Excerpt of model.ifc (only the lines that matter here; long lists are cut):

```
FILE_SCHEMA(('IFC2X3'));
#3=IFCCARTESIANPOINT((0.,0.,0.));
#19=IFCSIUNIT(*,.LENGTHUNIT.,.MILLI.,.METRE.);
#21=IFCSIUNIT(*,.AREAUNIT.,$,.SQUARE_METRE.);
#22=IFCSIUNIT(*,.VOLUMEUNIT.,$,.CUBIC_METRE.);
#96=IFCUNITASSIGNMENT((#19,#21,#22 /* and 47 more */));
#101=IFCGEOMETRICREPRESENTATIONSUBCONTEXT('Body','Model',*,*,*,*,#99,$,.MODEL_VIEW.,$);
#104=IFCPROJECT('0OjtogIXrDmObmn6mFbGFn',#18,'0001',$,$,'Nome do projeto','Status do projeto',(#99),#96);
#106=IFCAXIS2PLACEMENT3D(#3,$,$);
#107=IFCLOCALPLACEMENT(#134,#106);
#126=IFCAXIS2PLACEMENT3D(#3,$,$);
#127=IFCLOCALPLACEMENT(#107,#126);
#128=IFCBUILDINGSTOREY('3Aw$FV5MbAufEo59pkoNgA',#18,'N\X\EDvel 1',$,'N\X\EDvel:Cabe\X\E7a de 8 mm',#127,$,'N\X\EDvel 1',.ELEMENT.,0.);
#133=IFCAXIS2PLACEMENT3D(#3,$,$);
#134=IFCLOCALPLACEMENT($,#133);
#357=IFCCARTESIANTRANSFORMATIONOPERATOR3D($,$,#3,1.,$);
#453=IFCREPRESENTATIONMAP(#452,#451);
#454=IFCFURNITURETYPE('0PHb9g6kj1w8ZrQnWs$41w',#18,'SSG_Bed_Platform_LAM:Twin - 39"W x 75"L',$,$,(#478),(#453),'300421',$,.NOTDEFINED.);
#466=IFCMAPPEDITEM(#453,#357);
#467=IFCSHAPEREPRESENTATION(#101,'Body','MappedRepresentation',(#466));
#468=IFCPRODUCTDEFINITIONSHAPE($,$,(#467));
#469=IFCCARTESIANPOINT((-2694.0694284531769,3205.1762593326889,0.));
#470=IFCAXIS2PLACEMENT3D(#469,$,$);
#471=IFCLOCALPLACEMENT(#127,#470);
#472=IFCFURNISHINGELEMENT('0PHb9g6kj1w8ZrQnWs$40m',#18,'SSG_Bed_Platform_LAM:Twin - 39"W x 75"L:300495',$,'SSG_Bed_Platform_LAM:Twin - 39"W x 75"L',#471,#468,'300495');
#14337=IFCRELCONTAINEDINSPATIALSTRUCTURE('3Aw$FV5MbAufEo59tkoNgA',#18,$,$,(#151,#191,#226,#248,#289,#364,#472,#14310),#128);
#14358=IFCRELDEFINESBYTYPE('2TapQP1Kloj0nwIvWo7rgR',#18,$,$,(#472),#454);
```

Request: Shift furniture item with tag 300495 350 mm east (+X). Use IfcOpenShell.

```python
import ifcopenshell
import ifcopenshell.api.geometry
import ifcopenshell.util.placement
import ifcopenshell.util.unit

model = ifcopenshell.open("model.ifc")
unit_scale = ifcopenshell.util.unit.calculate_unit_scale(model)

item = model.by_id(472)
matrix = ifcopenshell.util.placement.get_local_placement(item.ObjectPlacement)
matrix[0, 3] += 0.35 / unit_scale
ifcopenshell.api.geometry.edit_object_placement(model, product=item, matrix=matrix, is_si=False)

print(ifcopenshell.util.placement.get_local_placement(item.ObjectPlacement).round(3) + 0.0)

model.write("model_rev.ifc")
```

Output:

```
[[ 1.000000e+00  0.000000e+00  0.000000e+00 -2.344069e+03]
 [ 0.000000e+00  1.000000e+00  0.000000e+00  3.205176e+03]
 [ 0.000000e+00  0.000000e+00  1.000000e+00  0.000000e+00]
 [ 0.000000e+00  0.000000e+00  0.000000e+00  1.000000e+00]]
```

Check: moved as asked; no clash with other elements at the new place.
